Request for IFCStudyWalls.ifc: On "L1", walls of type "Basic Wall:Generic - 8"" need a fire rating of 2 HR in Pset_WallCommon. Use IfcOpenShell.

First a look at what the model holds.

```python
import ifcopenshell
import ifcopenshell.util.element

model = ifcopenshell.open("IFCStudyWalls.ifc")
print(model.schema)
storey = next(s for s in model.by_type("IfcBuildingStorey") if s.Name == "L1")
walls = [e for e in ifcopenshell.util.element.get_decomposition(storey) if e.is_a("IfcWall")]
seen = {}
for e in walls:
    element_type = ifcopenshell.util.element.get_type(e)
    key = (element_type.Name if element_type != e and element_type else None, ifcopenshell.util.element.get_pset(e, "Pset_WallCommon", "FireRating"))
    seen[key] = seen.get(key, 0) + 1
for (name, value), count in sorted(seen.items(), key=str):
    print(count, "x", name, "|", value)
```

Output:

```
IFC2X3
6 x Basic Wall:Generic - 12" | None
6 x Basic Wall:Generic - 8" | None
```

```python
import ifcopenshell
import ifcopenshell.api.pset
import ifcopenshell.util.element

model = ifcopenshell.open("IFCStudyWalls.ifc")

storey = next(s for s in model.by_type("IfcBuildingStorey") if s.Name == "L1")
walls = [e for e in ifcopenshell.util.element.get_decomposition(storey) if e.is_a("IfcWall")]

count = 0
for e in walls:
    element_type = ifcopenshell.util.element.get_type(e)
    if element_type in (None, e) or element_type.Name != 'Basic Wall:Generic - 8"':
        continue
    # add_pset returns the element's existing set when there is one.
    pset = ifcopenshell.api.pset.add_pset(model, product=e, name="Pset_WallCommon")
    ifcopenshell.api.pset.edit_pset(model, pset=pset, properties={"FireRating": "2 HR"})
    count += 1

print(count, "walls updated")

model.write("IFCStudyWalls_v2.ifc")
```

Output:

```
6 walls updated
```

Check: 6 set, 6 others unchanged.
